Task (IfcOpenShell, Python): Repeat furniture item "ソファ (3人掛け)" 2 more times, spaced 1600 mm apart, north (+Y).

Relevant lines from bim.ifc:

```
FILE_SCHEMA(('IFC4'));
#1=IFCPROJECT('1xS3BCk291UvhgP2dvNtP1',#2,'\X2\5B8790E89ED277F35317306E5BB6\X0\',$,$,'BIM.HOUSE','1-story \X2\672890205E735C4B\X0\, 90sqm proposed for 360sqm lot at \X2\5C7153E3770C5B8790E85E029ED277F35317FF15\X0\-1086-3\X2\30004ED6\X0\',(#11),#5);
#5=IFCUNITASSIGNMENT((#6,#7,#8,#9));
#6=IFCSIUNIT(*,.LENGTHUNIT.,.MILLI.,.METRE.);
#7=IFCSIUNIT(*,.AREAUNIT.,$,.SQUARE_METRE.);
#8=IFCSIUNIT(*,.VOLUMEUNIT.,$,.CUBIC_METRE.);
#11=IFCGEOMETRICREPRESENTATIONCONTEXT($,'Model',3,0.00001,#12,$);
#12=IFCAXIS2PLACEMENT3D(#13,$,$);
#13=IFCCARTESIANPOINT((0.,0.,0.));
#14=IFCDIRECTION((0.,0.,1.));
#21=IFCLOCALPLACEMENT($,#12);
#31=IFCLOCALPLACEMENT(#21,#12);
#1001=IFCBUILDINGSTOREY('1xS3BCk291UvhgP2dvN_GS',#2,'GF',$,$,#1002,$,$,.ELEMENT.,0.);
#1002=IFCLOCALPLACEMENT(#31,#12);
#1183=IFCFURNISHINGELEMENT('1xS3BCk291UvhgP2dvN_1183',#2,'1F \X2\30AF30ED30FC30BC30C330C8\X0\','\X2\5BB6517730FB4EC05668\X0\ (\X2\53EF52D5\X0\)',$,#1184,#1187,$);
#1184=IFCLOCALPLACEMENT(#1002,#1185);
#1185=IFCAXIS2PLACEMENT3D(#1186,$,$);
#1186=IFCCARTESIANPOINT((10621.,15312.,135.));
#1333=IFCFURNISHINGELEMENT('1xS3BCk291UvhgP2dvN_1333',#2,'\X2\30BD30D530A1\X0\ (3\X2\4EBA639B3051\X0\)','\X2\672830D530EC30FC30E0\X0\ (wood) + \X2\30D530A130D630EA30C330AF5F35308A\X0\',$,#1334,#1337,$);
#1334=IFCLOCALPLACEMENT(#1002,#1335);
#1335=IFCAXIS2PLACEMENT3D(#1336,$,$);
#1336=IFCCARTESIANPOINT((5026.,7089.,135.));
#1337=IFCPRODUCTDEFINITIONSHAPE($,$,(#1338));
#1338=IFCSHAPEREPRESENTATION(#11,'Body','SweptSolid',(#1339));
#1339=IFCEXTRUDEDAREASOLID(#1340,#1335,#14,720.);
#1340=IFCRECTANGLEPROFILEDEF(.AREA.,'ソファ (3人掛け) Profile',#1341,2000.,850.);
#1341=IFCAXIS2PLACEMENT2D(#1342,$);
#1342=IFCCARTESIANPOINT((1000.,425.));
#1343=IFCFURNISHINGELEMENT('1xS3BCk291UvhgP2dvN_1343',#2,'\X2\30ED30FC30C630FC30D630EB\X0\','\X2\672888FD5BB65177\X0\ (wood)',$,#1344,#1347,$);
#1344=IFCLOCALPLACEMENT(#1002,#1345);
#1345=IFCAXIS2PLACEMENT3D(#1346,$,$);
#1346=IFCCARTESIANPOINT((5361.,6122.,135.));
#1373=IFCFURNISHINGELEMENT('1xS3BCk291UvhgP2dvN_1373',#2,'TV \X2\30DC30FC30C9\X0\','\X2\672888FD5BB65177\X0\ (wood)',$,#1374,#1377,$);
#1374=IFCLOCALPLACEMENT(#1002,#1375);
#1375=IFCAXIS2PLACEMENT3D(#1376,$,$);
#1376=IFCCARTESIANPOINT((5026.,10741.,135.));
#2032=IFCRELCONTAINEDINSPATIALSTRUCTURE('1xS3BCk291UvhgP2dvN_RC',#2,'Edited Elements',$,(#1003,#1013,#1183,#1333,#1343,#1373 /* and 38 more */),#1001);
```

```python
import numpy as np
import ifcopenshell
import ifcopenshell.api.geometry
import ifcopenshell.api.root
import ifcopenshell.util.element
import ifcopenshell.util.placement

model = ifcopenshell.open("bim.ifc")


def reuse_history(source, copy):
    """copy_class also copies each property set's owner history, people and application; keep the originals."""
    for rel in copy.IsDefinedBy:
        if rel.is_a("IfcRelDefinesByProperties") and (history := rel.RelatingPropertyDefinition.OwnerHistory):
            rel.RelatingPropertyDefinition.OwnerHistory = source.OwnerHistory
            ifcopenshell.util.element.remove_deep2(model, history)


source = model.by_guid("1xS3BCk291UvhgP2dvN_1333")
base = ifcopenshell.util.placement.get_local_placement(source.ObjectPlacement)
step = np.array([0.0, 1.0, 0.0]) * 1600.0

for i in range(1, 3):
    copy = ifcopenshell.api.root.copy_class(model, product=source)
    copy.Representation = ifcopenshell.util.element.copy_deep(
        model, source.Representation, exclude=["IfcGeometricRepresentationContext", "IfcRepresentationMap"]
    )
    reuse_history(source, copy)
    matrix = base.copy()
    matrix[:3, 3] += i * step
    print("added at", matrix[:3, 3].round(3) + 0.0)
    ifcopenshell.api.geometry.edit_object_placement(model, product=copy, matrix=matrix, is_si=False)

model.write("bim_v2.ifc")
```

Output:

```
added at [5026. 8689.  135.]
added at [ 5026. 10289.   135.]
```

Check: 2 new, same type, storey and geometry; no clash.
